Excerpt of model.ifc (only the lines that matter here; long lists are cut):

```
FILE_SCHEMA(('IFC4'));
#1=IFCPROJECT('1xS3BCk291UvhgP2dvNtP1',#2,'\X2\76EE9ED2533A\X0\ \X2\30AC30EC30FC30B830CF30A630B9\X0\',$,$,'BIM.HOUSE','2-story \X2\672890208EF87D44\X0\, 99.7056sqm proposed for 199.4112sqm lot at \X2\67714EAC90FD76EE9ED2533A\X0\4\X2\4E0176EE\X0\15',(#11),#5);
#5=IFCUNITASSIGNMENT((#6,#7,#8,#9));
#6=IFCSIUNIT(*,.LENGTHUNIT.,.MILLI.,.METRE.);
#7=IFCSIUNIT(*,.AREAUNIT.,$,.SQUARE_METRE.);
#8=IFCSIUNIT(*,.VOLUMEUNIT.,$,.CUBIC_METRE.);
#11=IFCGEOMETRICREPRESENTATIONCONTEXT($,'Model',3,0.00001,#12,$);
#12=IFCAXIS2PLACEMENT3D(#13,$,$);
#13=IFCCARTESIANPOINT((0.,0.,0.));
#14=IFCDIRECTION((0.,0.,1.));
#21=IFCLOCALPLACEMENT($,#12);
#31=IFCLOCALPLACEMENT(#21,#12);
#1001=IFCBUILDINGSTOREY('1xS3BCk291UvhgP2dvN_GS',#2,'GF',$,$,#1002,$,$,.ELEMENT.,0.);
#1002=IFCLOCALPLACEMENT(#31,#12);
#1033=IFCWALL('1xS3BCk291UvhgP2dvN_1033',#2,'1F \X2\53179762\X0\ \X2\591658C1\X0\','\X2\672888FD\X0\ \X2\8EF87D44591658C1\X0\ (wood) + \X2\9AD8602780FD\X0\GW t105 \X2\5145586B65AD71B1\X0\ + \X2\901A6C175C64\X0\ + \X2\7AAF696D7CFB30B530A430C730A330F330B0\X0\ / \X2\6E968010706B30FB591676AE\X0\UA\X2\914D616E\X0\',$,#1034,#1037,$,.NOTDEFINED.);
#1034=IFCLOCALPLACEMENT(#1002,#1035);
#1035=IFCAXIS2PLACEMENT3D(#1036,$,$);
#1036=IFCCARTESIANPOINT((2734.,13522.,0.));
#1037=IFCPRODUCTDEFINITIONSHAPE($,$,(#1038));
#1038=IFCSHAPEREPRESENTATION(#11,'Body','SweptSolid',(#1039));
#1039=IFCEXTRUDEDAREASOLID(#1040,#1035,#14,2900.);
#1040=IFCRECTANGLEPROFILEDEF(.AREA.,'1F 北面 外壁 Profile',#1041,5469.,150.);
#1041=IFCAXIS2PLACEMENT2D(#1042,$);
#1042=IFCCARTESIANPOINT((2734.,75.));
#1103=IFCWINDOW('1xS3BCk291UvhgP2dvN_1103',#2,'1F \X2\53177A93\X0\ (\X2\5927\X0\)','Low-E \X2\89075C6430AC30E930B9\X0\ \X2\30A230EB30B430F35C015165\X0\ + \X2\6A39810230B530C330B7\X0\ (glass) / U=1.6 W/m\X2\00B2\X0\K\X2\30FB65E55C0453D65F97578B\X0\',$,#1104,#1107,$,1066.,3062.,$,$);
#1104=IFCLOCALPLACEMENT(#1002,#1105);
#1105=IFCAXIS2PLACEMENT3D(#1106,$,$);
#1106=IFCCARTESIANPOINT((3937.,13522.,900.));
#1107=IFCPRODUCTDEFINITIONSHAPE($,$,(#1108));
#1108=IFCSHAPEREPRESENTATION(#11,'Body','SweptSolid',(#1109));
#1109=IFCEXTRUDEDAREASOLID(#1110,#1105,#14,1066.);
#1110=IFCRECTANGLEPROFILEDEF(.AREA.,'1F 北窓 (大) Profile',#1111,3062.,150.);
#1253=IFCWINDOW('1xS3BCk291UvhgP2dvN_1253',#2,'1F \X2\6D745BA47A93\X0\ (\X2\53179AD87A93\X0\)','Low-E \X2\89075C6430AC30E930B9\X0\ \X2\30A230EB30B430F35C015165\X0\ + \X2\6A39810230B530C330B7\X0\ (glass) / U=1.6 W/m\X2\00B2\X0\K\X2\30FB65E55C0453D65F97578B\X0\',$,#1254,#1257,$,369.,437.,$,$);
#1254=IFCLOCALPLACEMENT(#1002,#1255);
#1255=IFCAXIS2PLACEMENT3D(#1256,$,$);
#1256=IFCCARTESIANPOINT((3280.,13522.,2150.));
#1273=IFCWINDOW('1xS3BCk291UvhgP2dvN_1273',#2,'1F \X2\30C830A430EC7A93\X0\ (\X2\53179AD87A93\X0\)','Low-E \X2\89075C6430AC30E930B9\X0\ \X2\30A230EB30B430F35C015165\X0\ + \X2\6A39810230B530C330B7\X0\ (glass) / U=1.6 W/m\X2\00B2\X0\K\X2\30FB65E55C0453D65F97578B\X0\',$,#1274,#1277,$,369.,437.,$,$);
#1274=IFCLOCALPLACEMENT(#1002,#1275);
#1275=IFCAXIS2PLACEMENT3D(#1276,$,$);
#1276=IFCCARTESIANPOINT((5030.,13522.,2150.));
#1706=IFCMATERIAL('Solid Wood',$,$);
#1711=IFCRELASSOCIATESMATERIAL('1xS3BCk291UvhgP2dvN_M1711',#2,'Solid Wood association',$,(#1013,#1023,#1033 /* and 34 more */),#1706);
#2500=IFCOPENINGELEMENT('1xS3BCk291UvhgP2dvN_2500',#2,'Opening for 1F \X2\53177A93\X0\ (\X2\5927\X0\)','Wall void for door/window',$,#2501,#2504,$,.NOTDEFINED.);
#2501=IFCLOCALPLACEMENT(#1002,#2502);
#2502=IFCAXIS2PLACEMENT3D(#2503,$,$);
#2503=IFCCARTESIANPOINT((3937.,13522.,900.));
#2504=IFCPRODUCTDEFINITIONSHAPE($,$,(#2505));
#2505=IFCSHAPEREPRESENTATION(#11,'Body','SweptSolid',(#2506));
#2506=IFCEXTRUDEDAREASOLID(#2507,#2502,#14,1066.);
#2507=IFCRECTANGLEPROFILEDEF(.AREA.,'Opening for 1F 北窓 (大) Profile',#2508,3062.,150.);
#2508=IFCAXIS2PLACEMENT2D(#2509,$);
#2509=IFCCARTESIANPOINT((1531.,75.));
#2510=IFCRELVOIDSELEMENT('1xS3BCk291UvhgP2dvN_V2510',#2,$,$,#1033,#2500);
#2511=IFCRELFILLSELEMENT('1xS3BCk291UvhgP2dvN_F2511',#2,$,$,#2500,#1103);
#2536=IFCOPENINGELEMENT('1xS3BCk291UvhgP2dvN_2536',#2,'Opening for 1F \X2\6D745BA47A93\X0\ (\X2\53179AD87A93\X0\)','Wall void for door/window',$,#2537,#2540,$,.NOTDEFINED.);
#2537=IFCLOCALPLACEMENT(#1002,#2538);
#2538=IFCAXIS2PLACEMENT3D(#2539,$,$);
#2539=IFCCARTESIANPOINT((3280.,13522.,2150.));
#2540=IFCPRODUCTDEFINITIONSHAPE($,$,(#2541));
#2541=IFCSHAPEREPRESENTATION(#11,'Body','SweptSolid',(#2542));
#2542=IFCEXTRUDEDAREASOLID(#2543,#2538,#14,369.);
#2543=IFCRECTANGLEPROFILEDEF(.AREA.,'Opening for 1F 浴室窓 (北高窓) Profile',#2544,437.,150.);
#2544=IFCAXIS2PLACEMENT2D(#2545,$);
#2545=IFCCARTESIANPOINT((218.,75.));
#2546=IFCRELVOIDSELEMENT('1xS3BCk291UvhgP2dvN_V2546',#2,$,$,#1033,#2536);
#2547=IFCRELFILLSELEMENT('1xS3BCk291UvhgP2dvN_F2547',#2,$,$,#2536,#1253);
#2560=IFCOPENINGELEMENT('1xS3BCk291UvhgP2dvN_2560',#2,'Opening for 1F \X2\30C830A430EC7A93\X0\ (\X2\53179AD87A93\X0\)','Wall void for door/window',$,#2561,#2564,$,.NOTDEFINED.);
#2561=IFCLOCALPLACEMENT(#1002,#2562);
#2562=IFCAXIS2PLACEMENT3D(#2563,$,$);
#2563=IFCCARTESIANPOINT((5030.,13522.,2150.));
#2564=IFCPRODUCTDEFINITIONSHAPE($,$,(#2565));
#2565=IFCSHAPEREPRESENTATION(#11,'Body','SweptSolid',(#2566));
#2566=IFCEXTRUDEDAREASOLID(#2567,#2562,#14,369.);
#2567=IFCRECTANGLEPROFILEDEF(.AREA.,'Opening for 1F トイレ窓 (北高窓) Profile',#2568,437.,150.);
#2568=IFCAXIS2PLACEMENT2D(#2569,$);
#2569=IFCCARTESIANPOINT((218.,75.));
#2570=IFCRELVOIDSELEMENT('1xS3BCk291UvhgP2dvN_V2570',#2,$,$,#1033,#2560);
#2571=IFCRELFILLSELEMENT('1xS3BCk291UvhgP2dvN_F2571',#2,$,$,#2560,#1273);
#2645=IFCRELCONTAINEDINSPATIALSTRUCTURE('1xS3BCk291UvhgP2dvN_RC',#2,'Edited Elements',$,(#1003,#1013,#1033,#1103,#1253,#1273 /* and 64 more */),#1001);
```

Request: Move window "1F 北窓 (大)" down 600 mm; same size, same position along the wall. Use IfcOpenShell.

```python
import numpy as np
import ifcopenshell
import ifcopenshell.api.geometry
import ifcopenshell.util.placement
import ifcopenshell.util.unit

model = ifcopenshell.open("model.ifc")
unit_scale = ifcopenshell.util.unit.calculate_unit_scale(model)

window = model.by_guid("1xS3BCk291UvhgP2dvN_1103")
opening = window.FillsVoids[0].RelatingOpeningElement
dz = -0.6 / unit_scale

shift = np.array([0.0, 0.0, dz])
# The window is not placed relative to its opening, so move both.
for product in (opening, window):
    matrix = ifcopenshell.util.placement.get_local_placement(product.ObjectPlacement)
    matrix[:3, 3] += shift
    ifcopenshell.api.geometry.edit_object_placement(model, product=product, matrix=matrix, is_si=False)

print(f"moved by {dz * unit_scale:+.3f} m")

model.write("model_edited.ifc")
```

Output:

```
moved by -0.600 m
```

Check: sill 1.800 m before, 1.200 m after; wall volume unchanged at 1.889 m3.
